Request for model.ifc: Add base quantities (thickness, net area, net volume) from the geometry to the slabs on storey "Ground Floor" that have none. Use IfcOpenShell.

First a look at what the model holds.

```python
import ifcopenshell
import ifcopenshell.util.element
import ifcopenshell.util.unit

model = ifcopenshell.open("model.ifc")
print(model.schema)
for unit_type in ("LENGTHUNIT", "AREAUNIT", "VOLUMEUNIT"):
    print(unit_type, ifcopenshell.util.unit.calculate_unit_scale(model, unit_type))
storey = next(s for s in model.by_type("IfcBuildingStorey") if s.Name == "Ground Floor")
slabs = [e for e in ifcopenshell.util.element.get_decomposition(storey) if e.is_a("IfcSlab")]
for e in sorted(slabs, key=lambda e: e.id()):
    print(e.id(), e.is_a(), e.Name, list(ifcopenshell.util.element.get_psets(e, qtos_only=True)), sep=" | ")
```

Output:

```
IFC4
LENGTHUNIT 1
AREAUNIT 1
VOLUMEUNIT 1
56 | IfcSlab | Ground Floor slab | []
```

```python
import ifcopenshell
import ifcopenshell.api.pset
import ifcopenshell.geom
import ifcopenshell.util.element
import ifcopenshell.util.shape
import ifcopenshell.util.unit

model = ifcopenshell.open("model.ifc")
unit_scale = ifcopenshell.util.unit.calculate_unit_scale(model)
area_scale = ifcopenshell.util.unit.calculate_unit_scale(model, "AREAUNIT")
volume_scale = ifcopenshell.util.unit.calculate_unit_scale(model, "VOLUMEUNIT")
settings = ifcopenshell.geom.settings()

storey = next(s for s in model.by_type("IfcBuildingStorey") if s.Name == "Ground Floor")
slabs = [e for e in ifcopenshell.util.element.get_decomposition(storey) if e.is_a("IfcSlab")]

for e in sorted(slabs, key=lambda e: e.id()):
    if ifcopenshell.util.element.get_psets(e, qtos_only=True, should_inherit=False):
        continue
    # Geometry comes back in metres, in the element's own axes.
    shape = ifcopenshell.geom.create_shape(settings, e)
    values = {
        "Width": ifcopenshell.util.shape.get_z(shape.geometry) / unit_scale,
        "NetArea": ifcopenshell.util.shape.get_footprint_area(shape.geometry) / area_scale,
        "NetVolume": ifcopenshell.util.shape.get_volume(shape.geometry) / volume_scale,
    }
    qto = ifcopenshell.api.pset.add_qto(model, product=e, name="Qto_SlabBaseQuantities")
    ifcopenshell.api.pset.edit_qto(model, qto=qto, properties=values)
    print(e.id(), {k: round(v, 3) for k, v in values.items()})

model.write("model_updated.ifc")
```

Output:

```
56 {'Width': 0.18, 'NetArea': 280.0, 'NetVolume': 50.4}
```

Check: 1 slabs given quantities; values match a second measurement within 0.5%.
